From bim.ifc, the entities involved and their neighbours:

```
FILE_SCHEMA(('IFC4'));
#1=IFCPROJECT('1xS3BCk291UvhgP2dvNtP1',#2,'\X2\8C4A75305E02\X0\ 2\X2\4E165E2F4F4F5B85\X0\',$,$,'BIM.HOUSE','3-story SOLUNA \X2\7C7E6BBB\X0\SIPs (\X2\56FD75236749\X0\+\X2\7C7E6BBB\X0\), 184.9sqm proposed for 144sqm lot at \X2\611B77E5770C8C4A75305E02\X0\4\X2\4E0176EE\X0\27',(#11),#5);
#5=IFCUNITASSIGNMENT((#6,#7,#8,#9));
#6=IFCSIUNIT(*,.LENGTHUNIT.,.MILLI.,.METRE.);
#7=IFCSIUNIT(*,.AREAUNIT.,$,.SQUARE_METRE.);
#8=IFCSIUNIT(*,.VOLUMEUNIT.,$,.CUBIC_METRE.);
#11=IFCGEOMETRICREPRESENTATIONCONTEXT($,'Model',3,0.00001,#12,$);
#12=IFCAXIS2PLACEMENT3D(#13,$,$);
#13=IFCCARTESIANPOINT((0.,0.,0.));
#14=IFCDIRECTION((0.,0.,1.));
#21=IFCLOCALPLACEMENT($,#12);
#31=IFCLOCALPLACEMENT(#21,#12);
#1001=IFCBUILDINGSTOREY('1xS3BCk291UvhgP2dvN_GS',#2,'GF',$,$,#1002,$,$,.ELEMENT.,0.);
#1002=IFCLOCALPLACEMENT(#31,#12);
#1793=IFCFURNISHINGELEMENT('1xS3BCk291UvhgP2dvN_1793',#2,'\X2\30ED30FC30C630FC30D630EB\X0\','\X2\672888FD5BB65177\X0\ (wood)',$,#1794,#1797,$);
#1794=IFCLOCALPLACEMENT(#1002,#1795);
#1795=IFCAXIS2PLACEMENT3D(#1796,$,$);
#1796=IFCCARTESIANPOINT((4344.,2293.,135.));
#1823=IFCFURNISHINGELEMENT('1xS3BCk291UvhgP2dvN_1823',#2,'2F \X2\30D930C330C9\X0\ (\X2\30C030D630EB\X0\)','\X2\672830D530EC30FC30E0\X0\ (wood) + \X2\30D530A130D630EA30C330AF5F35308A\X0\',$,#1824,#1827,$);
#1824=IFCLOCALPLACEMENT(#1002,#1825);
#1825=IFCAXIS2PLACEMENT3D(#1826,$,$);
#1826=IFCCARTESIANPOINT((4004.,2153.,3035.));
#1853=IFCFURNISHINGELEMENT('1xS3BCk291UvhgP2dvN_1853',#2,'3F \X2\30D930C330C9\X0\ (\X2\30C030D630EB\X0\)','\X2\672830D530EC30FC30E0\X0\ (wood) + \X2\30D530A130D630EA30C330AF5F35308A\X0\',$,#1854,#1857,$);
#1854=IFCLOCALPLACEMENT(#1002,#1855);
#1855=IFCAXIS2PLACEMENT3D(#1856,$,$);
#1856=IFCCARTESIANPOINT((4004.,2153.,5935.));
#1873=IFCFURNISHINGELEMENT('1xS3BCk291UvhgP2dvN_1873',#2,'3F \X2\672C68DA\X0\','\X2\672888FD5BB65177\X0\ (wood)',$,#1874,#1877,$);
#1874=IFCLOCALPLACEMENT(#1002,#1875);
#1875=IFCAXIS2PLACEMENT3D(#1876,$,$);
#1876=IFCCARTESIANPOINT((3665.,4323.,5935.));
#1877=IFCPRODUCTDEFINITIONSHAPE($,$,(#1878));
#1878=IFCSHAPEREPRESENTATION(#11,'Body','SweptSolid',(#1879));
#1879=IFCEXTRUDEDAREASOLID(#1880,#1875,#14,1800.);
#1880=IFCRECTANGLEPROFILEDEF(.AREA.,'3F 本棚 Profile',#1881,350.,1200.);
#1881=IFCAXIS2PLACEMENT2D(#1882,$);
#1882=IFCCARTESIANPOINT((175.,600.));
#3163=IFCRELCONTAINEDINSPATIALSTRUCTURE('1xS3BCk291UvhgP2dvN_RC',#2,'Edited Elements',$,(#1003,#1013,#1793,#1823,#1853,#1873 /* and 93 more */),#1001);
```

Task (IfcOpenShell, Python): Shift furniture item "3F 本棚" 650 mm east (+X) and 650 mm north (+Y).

```python
import ifcopenshell
import ifcopenshell.api.geometry
import ifcopenshell.util.placement

model = ifcopenshell.open("bim.ifc")

item = model.by_guid("1xS3BCk291UvhgP2dvN_1873")
matrix = ifcopenshell.util.placement.get_local_placement(item.ObjectPlacement)
matrix[0, 3] += 650.0
matrix[1, 3] += 650.0
ifcopenshell.api.geometry.edit_object_placement(model, product=item, matrix=matrix, is_si=False)

print(ifcopenshell.util.placement.get_local_placement(item.ObjectPlacement).round(3) + 0.0)

model.write("bim_updated.ifc")
```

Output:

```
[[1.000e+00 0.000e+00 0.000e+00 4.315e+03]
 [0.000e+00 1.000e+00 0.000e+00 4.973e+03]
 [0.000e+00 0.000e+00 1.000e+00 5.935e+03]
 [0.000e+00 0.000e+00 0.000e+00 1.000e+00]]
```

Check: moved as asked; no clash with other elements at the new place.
